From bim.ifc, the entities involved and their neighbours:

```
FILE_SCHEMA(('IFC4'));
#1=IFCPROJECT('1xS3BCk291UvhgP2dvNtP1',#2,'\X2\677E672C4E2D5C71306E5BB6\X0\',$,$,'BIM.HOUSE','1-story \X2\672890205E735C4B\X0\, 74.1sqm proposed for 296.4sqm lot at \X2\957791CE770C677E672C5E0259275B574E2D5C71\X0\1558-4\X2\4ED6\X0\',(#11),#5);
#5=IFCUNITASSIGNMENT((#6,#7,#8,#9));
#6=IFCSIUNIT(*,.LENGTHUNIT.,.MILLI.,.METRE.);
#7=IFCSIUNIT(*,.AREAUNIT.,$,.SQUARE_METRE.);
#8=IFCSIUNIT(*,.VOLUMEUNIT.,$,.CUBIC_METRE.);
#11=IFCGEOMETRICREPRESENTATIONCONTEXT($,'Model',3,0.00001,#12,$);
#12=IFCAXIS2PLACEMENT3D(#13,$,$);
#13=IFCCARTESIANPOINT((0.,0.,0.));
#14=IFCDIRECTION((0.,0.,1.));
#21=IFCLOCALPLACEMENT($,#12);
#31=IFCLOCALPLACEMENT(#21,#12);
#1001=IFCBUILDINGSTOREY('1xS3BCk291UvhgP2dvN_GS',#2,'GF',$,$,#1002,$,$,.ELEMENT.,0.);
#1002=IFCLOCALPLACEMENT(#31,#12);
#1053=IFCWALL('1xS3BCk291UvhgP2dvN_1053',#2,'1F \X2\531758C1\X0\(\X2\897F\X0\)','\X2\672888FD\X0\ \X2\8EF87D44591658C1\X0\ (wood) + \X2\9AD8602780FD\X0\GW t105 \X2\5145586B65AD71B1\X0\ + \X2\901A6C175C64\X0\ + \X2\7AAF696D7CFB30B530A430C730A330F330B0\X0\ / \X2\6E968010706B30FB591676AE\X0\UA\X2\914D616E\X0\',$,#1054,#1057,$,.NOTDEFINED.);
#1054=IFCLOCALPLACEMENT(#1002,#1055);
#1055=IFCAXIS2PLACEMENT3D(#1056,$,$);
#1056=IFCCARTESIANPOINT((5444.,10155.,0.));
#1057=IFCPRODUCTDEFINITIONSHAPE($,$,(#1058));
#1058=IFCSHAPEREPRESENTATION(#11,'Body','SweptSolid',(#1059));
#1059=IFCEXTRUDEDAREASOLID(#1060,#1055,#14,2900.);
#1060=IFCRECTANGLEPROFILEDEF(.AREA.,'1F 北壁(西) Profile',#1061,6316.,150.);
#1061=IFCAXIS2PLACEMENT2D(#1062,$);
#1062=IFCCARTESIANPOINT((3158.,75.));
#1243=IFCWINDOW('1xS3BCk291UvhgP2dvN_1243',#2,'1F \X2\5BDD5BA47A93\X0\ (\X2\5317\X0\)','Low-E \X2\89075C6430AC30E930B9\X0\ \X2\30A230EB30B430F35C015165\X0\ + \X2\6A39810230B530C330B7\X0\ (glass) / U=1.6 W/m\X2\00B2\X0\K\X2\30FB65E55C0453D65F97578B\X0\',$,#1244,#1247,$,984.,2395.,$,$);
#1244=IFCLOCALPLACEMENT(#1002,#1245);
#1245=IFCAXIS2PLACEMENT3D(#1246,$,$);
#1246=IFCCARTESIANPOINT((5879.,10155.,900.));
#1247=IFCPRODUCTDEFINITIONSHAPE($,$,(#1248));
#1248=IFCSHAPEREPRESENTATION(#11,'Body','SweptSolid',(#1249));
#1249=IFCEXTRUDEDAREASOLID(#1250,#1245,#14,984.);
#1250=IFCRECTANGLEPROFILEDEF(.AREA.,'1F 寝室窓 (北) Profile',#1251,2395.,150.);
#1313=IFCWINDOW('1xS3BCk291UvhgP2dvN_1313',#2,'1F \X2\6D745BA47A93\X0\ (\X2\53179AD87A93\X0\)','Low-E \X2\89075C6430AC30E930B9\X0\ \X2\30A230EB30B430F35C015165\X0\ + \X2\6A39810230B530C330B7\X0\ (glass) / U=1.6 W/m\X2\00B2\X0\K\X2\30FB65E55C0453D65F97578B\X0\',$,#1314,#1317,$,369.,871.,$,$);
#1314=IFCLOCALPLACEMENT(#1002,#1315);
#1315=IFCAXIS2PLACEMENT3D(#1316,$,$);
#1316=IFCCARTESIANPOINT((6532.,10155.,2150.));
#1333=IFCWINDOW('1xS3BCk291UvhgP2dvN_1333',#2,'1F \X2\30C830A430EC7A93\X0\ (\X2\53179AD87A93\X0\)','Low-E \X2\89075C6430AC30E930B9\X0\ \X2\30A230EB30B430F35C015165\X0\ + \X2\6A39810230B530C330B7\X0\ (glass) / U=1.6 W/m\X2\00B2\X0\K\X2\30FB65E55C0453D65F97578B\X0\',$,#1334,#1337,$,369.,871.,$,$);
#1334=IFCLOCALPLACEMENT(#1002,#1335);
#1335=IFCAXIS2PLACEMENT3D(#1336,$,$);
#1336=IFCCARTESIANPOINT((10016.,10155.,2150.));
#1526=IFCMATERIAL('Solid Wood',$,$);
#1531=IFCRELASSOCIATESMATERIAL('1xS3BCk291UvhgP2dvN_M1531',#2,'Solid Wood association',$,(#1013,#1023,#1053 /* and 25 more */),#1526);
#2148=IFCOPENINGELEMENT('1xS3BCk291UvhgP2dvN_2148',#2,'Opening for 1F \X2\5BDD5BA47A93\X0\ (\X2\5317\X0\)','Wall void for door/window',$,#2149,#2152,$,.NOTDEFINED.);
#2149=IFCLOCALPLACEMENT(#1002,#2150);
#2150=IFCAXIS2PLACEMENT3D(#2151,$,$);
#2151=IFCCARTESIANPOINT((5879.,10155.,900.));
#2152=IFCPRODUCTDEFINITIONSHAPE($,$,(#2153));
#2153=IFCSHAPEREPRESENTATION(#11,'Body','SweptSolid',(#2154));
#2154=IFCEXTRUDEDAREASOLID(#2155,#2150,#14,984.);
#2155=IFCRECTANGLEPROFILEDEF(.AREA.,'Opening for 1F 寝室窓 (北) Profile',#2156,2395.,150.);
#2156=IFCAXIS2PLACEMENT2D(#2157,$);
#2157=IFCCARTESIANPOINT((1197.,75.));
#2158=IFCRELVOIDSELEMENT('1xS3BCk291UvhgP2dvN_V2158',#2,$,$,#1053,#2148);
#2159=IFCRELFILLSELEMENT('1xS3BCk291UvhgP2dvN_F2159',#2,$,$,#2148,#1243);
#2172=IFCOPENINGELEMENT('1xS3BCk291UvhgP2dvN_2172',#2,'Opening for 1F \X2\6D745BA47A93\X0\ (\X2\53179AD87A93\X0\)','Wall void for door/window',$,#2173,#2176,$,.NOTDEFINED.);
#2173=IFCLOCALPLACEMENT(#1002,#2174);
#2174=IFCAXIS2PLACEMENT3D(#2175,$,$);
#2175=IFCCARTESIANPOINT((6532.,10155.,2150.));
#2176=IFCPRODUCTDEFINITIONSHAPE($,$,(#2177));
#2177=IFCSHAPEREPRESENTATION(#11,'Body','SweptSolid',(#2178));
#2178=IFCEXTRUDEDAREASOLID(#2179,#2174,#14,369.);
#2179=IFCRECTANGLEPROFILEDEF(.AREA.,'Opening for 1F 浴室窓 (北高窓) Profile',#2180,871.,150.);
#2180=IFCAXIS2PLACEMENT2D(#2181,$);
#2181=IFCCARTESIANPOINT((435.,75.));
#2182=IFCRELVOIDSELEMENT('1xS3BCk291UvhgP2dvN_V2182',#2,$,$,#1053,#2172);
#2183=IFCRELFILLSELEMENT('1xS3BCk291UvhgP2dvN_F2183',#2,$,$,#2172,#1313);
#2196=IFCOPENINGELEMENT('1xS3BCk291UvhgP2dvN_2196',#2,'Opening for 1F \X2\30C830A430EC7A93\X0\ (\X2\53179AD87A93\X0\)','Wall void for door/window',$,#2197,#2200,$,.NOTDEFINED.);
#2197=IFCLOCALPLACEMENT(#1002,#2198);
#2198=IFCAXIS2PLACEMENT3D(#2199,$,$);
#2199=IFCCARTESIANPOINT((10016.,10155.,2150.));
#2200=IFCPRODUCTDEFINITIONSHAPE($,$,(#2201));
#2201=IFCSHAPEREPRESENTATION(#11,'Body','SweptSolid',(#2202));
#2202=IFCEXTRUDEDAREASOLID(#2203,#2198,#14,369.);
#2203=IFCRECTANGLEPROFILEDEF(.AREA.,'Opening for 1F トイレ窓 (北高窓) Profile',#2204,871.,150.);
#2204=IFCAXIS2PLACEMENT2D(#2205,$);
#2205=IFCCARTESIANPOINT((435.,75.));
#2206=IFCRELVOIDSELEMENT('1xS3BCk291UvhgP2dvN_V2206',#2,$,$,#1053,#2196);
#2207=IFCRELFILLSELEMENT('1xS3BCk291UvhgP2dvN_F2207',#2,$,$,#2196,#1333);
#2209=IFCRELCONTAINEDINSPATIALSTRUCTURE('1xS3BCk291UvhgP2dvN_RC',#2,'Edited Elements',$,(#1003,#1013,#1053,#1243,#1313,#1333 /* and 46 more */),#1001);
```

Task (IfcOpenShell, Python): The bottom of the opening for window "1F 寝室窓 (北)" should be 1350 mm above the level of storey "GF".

```python
import numpy as np
import ifcopenshell
import ifcopenshell.api.geometry
import ifcopenshell.geom
import ifcopenshell.util.element
import ifcopenshell.util.placement
import ifcopenshell.util.shape
import ifcopenshell.util.unit

model = ifcopenshell.open("bim.ifc")
unit_scale = ifcopenshell.util.unit.calculate_unit_scale(model)

window = model.by_guid("1xS3BCk291UvhgP2dvN_1243")
opening = window.FillsVoids[0].RelatingOpeningElement
storey = ifcopenshell.util.element.get_container(window, ifc_class="IfcBuildingStorey")
level = ifcopenshell.util.placement.get_local_placement(storey.ObjectPlacement)[2, 3]

# The opening's origin need not be at the sill, so measure its lowest point.
shape = ifcopenshell.geom.create_shape(ifcopenshell.geom.settings(), opening)
bottom = ifcopenshell.util.shape.get_shape_bottom_elevation(shape, shape.geometry) / unit_scale
dz = level + 1350.0 - bottom

shift = np.array([0.0, 0.0, dz])
# The window is not placed relative to its opening, so move both.
for product in (opening, window):
    matrix = ifcopenshell.util.placement.get_local_placement(product.ObjectPlacement)
    matrix[:3, 3] += shift
    ifcopenshell.api.geometry.edit_object_placement(model, product=product, matrix=matrix, is_si=False)

print(f"moved by {dz * unit_scale:+.3f} m")

model.write("bim-out.ifc")
```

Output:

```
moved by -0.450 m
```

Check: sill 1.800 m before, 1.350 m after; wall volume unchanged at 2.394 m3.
